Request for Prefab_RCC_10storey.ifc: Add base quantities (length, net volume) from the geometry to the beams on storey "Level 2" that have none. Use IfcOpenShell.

First a look at what the model holds.

```python
import ifcopenshell
import ifcopenshell.util.element
import ifcopenshell.util.unit

model = ifcopenshell.open("Prefab_RCC_10storey.ifc")
print(model.schema)
for unit_type in ("LENGTHUNIT", "AREAUNIT", "VOLUMEUNIT"):
    print(unit_type, ifcopenshell.util.unit.calculate_unit_scale(model, unit_type))
storey = next(s for s in model.by_type("IfcBuildingStorey") if s.Name == "Level 2")
beams = [e for e in ifcopenshell.util.element.get_decomposition(storey) if e.is_a("IfcBeam")]
for e in sorted(beams, key=lambda e: e.id()):
    print(e.id(), e.is_a(), e.Name, list(ifcopenshell.util.element.get_psets(e, qtos_only=True)), sep=" | ")
```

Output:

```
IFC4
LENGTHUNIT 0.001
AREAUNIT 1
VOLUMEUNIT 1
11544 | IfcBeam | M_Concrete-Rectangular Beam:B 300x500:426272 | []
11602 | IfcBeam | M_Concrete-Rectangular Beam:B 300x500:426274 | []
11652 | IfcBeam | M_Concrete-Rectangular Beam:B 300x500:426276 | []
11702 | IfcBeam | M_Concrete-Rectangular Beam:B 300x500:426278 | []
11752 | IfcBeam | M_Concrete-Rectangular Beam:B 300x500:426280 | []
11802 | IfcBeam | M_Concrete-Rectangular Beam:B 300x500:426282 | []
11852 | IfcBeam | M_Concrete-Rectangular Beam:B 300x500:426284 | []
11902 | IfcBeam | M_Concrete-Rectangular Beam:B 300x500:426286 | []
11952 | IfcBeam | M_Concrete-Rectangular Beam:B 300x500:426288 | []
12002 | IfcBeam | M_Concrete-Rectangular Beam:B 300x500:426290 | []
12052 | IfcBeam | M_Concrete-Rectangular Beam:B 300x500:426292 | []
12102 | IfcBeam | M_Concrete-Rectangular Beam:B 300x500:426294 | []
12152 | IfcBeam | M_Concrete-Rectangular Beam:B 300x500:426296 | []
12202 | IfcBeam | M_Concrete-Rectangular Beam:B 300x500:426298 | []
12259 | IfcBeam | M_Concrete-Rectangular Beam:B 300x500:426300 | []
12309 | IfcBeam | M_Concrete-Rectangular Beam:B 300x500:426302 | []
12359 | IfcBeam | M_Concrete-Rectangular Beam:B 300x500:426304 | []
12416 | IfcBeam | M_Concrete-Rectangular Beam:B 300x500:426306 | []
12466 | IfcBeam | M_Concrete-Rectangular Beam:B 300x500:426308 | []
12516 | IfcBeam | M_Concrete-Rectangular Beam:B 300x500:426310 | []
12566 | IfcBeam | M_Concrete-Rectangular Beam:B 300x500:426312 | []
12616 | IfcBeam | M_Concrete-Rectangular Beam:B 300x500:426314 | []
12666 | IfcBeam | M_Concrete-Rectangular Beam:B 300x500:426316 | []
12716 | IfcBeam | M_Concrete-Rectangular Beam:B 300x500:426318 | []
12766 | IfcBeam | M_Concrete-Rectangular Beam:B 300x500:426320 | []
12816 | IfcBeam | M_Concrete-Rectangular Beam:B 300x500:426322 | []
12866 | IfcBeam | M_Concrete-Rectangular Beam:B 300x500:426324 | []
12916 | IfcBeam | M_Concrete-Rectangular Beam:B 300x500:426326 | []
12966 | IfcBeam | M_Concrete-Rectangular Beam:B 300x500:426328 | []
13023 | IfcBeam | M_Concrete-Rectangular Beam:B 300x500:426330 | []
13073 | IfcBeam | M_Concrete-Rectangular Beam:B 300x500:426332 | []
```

```python
import ifcopenshell
import ifcopenshell.api.pset
import ifcopenshell.geom
import ifcopenshell.util.element
import ifcopenshell.util.shape
import ifcopenshell.util.unit

model = ifcopenshell.open("Prefab_RCC_10storey.ifc")
unit_scale = ifcopenshell.util.unit.calculate_unit_scale(model)
volume_scale = ifcopenshell.util.unit.calculate_unit_scale(model, "VOLUMEUNIT")
settings = ifcopenshell.geom.settings()

storey = next(s for s in model.by_type("IfcBuildingStorey") if s.Name == "Level 2")
beams = [e for e in ifcopenshell.util.element.get_decomposition(storey) if e.is_a("IfcBeam")]

for e in sorted(beams, key=lambda e: e.id()):
    if ifcopenshell.util.element.get_psets(e, qtos_only=True, should_inherit=False):
        continue
    # Geometry comes back in metres, in the element's own axes.
    shape = ifcopenshell.geom.create_shape(settings, e)
    values = {
        "Length": ifcopenshell.util.shape.get_max_xyz(shape.geometry) / unit_scale,
        "NetVolume": ifcopenshell.util.shape.get_volume(shape.geometry) / volume_scale,
    }
    qto = ifcopenshell.api.pset.add_qto(model, product=e, name="Qto_BeamBaseQuantities")
    ifcopenshell.api.pset.edit_qto(model, qto=qto, properties=values)
    print(e.id(), {k: round(v, 3) for k, v in values.items()})

model.write("Prefab_RCC_10storey_updated.ifc")
```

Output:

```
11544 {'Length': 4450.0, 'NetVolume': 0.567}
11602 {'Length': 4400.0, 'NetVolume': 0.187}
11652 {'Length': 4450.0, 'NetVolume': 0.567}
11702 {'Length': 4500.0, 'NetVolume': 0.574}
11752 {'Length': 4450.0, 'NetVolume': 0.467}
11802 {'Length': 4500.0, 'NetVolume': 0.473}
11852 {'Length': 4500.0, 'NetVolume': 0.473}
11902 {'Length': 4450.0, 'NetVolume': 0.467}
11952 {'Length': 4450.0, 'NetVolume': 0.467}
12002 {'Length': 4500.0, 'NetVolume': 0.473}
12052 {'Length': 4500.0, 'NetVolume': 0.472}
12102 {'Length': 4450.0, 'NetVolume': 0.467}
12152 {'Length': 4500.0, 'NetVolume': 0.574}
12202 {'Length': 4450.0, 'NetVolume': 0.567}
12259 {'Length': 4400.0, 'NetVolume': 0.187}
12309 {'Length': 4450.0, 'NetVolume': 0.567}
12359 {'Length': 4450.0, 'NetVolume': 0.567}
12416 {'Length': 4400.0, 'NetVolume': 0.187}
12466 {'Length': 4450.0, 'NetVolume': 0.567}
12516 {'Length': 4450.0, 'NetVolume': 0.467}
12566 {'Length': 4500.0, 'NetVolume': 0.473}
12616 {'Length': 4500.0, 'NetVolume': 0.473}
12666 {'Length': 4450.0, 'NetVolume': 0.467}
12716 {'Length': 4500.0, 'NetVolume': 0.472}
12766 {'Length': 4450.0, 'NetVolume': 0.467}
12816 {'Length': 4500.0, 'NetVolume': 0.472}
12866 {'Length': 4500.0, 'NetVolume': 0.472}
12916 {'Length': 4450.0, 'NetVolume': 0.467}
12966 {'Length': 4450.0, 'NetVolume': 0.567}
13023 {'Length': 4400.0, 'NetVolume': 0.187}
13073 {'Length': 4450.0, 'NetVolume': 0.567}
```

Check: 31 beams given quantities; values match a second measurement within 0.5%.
